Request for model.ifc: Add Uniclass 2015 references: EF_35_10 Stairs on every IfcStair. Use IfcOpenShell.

First a look at what the model holds.

```python
import ifcopenshell

model = ifcopenshell.open("model.ifc")
print(model.schema)
print("classifications:", [c.Name for c in model.by_type("IfcClassification")])
for ifc_class in ("IfcDoor", "IfcRoof", "IfcStair", "IfcWall", "IfcWindow"):
    print(ifc_class, len(model.by_type(ifc_class)))
```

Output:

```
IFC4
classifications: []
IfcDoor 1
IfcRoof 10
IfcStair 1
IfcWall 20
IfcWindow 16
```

```python
import ifcopenshell
import ifcopenshell.api.classification

model = ifcopenshell.open("model.ifc")

system = ifcopenshell.api.classification.add_classification(model, classification="Uniclass 2015")

codes = {
    "IfcStair": ("EF_35_10", "Stairs"),
}
for ifc_class, (code, name) in codes.items():
    products = model.by_type(ifc_class)
    ifcopenshell.api.classification.add_reference(
        model, products=products, classification=system, identification=code, name=name
    )
    print(code, len(products))

model.write("model-out.ifc")
```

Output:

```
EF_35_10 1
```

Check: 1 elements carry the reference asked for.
